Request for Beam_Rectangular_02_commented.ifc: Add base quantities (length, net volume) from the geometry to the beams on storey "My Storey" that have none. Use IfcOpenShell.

First a look at what the model holds.

```python
import ifcopenshell
import ifcopenshell.util.element
import ifcopenshell.util.unit

model = ifcopenshell.open("Beam_Rectangular_02_commented.ifc")
print(model.schema)
for unit_type in ("LENGTHUNIT", "AREAUNIT", "VOLUMEUNIT"):
    print(unit_type, ifcopenshell.util.unit.calculate_unit_scale(model, unit_type))
storey = next(s for s in model.by_type("IfcBuildingStorey") if s.Name == "My Storey")
beams = [e for e in ifcopenshell.util.element.get_decomposition(storey) if e.is_a("IfcBeam")]
for e in sorted(beams, key=lambda e: e.id()):
    print(e.id(), e.is_a(), e.Name, list(ifcopenshell.util.element.get_psets(e, qtos_only=True)), sep=" | ")
```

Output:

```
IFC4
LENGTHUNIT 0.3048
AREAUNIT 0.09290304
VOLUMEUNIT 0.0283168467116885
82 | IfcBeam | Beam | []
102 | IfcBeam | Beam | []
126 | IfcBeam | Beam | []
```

```python
import ifcopenshell
import ifcopenshell.api.pset
import ifcopenshell.geom
import ifcopenshell.util.element
import ifcopenshell.util.shape
import ifcopenshell.util.unit

model = ifcopenshell.open("Beam_Rectangular_02_commented.ifc")
unit_scale = ifcopenshell.util.unit.calculate_unit_scale(model)
volume_scale = ifcopenshell.util.unit.calculate_unit_scale(model, "VOLUMEUNIT")
settings = ifcopenshell.geom.settings()

storey = next(s for s in model.by_type("IfcBuildingStorey") if s.Name == "My Storey")
beams = [e for e in ifcopenshell.util.element.get_decomposition(storey) if e.is_a("IfcBeam")]

for e in sorted(beams, key=lambda e: e.id()):
    if ifcopenshell.util.element.get_psets(e, qtos_only=True, should_inherit=False):
        continue
    # Geometry comes back in metres, in the element's own axes.
    shape = ifcopenshell.geom.create_shape(settings, e)
    values = {
        "Length": ifcopenshell.util.shape.get_max_xyz(shape.geometry) / unit_scale,
        "NetVolume": ifcopenshell.util.shape.get_volume(shape.geometry) / volume_scale,
    }
    qto = ifcopenshell.api.pset.add_qto(model, product=e, name="Qto_BeamBaseQuantities")
    ifcopenshell.api.pset.edit_qto(model, qto=qto, properties=values)
    print(e.id(), {k: round(v, 3) for k, v in values.items()})

model.write("Beam_Rectangular_02_commented-out.ifc")
```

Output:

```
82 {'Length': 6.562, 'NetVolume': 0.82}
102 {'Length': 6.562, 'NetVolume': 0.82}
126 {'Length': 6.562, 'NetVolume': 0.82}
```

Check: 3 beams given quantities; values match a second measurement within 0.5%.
